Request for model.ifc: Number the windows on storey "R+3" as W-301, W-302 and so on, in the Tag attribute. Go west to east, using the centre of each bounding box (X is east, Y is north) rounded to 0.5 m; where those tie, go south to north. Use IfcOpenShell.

First a look at what the model holds.

```python
import ifcopenshell
import ifcopenshell.util.element
import ifcopenshell.util.placement

model = ifcopenshell.open("model.ifc")
print(model.schema)
storey = next(s for s in model.by_type("IfcBuildingStorey") if s.Name == "R+3")
windows = [e for e in ifcopenshell.util.element.get_decomposition(storey) if e.is_a("IfcWindow")]
for e in sorted(windows, key=lambda e: e.id()):
    origin = ifcopenshell.util.placement.get_local_placement(e.ObjectPlacement)[:3, 3]
    print(e.id(), e.Tag, e.Name, origin.round(2) + 0.0, sep=" | ")
```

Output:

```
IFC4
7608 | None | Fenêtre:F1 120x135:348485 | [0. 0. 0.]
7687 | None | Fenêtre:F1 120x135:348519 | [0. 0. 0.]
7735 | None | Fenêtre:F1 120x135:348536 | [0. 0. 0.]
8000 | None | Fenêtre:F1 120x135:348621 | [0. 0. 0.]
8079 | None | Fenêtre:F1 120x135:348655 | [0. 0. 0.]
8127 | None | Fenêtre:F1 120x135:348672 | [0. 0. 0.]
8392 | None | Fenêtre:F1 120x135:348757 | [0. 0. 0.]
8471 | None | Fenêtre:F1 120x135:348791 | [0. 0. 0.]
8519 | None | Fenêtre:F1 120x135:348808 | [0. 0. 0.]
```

```python
import ifcopenshell
import ifcopenshell.geom
import ifcopenshell.util.element
import ifcopenshell.util.shape

model = ifcopenshell.open("model.ifc")
settings = ifcopenshell.geom.settings()
settings.set("use-world-coords", True)


def centre(element):
    shape = ifcopenshell.geom.create_shape(settings, element)
    return ifcopenshell.util.shape.get_bbox_centroid(shape.geometry)


storey = next(s for s in model.by_type("IfcBuildingStorey") if s.Name == "R+3")
windows = [e for e in ifcopenshell.util.element.get_decomposition(storey) if e.is_a("IfcWindow")]

# Insertion points can sit at a corner or the storey origin, so sort by the geometry (in metres).
centres = {e: centre(e) for e in windows}
windows.sort(key=lambda e: (round(centres[e][0] / 0.5), centres[e][1]))

for i, e in enumerate(windows, start=1):
    number = f"W-3{i:02d}"
    e.Tag = number
    print(e.id(), number)

model.write("model_edited.ifc")
```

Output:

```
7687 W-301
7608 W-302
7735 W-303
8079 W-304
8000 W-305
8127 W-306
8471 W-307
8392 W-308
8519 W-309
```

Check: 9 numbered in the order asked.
